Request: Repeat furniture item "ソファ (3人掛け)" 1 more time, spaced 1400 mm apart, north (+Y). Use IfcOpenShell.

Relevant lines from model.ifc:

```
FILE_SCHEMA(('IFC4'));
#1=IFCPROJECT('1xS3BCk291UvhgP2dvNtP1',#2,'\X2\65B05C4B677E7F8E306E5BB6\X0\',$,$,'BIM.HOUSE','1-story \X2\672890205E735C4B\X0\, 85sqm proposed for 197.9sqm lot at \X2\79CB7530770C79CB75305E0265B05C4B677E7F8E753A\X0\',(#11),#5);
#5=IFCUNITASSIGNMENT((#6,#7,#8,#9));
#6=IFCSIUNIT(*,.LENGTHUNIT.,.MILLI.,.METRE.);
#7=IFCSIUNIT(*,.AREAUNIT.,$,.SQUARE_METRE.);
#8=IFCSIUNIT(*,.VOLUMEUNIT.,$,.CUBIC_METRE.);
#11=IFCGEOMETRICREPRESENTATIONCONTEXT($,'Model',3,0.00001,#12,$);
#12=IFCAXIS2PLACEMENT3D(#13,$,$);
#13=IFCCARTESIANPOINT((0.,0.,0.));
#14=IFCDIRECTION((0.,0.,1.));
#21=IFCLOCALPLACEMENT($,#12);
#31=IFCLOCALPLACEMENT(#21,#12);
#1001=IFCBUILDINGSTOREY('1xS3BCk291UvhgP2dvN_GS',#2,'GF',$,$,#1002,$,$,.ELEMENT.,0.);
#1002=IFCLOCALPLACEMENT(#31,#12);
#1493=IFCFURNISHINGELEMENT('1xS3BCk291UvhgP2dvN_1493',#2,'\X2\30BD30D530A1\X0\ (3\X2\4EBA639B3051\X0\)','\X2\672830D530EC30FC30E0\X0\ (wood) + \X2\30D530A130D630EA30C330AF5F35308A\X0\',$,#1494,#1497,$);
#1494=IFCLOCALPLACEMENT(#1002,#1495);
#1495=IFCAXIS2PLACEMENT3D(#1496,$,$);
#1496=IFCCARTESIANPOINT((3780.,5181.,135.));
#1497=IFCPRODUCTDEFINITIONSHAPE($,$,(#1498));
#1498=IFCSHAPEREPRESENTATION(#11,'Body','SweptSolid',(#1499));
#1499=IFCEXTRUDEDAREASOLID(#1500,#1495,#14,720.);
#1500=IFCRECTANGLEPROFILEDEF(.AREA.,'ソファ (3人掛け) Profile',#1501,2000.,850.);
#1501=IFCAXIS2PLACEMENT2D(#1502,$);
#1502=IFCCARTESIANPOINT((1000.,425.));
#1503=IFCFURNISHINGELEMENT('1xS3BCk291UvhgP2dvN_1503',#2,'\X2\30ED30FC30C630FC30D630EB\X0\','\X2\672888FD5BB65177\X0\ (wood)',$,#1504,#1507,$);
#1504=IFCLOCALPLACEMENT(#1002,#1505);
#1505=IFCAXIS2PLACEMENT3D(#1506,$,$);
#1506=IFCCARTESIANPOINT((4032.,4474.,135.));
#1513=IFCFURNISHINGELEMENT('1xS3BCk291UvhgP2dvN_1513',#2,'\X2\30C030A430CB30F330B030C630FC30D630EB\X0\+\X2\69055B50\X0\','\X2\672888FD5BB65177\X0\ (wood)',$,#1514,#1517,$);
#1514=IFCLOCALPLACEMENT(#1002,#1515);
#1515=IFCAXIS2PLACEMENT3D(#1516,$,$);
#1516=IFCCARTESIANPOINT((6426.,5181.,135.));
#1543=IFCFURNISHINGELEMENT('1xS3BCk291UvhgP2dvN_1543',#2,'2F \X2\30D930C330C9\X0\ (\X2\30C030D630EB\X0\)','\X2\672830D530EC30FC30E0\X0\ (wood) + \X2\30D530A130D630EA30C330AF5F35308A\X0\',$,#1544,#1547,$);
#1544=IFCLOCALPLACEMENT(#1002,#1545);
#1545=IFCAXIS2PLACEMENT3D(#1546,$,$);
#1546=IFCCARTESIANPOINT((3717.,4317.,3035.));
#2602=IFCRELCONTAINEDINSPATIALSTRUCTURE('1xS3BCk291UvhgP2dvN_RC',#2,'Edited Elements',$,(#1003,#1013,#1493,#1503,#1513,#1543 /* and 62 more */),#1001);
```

```python
import numpy as np
import ifcopenshell
import ifcopenshell.api.geometry
import ifcopenshell.api.root
import ifcopenshell.util.element
import ifcopenshell.util.placement

model = ifcopenshell.open("model.ifc")


def reuse_history(source, copy):
    """copy_class also copies each property set's owner history, people and application; keep the originals."""
    for rel in copy.IsDefinedBy:
        if rel.is_a("IfcRelDefinesByProperties") and (history := rel.RelatingPropertyDefinition.OwnerHistory):
            rel.RelatingPropertyDefinition.OwnerHistory = source.OwnerHistory
            ifcopenshell.util.element.remove_deep2(model, history)


source = model.by_guid("1xS3BCk291UvhgP2dvN_1493")
base = ifcopenshell.util.placement.get_local_placement(source.ObjectPlacement)
step = np.array([0.0, 1.0, 0.0]) * 1400.0

for i in range(1, 2):
    copy = ifcopenshell.api.root.copy_class(model, product=source)
    copy.Representation = ifcopenshell.util.element.copy_deep(
        model, source.Representation, exclude=["IfcGeometricRepresentationContext", "IfcRepresentationMap"]
    )
    reuse_history(source, copy)
    matrix = base.copy()
    matrix[:3, 3] += i * step
    print("added at", matrix[:3, 3].round(3) + 0.0)
    ifcopenshell.api.geometry.edit_object_placement(model, product=copy, matrix=matrix, is_si=False)

model.write("model_v2.ifc")
```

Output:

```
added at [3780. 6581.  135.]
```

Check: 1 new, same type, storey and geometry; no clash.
